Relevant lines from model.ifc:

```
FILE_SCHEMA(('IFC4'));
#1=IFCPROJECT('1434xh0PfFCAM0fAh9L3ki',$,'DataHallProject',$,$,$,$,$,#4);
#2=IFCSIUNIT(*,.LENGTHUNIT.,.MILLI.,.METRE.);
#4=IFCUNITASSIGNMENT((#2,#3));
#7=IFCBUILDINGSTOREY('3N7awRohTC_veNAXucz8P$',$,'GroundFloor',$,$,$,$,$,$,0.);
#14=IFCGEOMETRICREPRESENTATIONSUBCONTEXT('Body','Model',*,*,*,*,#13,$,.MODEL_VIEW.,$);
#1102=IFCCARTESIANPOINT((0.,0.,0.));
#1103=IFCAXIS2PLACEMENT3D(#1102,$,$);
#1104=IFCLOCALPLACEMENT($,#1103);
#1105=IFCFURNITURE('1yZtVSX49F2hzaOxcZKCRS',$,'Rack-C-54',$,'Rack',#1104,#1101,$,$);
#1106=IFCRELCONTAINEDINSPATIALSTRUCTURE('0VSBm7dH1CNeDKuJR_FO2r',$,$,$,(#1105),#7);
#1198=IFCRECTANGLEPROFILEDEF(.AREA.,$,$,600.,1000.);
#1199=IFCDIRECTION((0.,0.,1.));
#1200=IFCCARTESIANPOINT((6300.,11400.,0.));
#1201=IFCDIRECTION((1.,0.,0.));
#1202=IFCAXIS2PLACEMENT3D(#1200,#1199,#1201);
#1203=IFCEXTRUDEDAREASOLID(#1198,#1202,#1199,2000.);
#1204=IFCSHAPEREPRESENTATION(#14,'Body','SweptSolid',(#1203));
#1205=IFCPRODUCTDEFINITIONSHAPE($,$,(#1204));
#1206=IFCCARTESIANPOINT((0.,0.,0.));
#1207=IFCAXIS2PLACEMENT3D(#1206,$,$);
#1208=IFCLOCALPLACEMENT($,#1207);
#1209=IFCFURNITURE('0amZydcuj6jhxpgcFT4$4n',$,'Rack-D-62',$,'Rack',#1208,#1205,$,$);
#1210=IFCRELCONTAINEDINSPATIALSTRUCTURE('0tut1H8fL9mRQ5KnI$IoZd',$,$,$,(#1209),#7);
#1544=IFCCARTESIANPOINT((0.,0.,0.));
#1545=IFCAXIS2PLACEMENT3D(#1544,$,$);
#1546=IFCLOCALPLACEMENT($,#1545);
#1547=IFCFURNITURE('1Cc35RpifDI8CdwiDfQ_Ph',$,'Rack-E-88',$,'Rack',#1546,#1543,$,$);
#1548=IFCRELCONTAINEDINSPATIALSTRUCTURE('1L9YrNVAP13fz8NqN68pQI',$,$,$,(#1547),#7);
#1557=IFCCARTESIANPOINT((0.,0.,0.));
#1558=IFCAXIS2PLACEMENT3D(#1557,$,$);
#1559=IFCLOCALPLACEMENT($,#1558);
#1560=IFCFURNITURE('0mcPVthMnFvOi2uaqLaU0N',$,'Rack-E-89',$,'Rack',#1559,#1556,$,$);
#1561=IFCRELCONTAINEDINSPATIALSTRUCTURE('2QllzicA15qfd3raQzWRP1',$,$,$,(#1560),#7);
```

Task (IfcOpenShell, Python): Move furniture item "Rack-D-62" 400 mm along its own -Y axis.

```python
import ifcopenshell
import ifcopenshell.api.geometry
import ifcopenshell.util.placement
import ifcopenshell.util.unit

model = ifcopenshell.open("model.ifc")
unit_scale = ifcopenshell.util.unit.calculate_unit_scale(model)

item = model.by_guid("0amZydcuj6jhxpgcFT4$4n")
matrix = ifcopenshell.util.placement.get_local_placement(item.ObjectPlacement)
matrix[:3, 3] -= matrix[:3, 1] * 0.4 / unit_scale
ifcopenshell.api.geometry.edit_object_placement(model, product=item, matrix=matrix, is_si=False)

print(ifcopenshell.util.placement.get_local_placement(item.ObjectPlacement).round(3) + 0.0)

model.write("model_edited.ifc")
```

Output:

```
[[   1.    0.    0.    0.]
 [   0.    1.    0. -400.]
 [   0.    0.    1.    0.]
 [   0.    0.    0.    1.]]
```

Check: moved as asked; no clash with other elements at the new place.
